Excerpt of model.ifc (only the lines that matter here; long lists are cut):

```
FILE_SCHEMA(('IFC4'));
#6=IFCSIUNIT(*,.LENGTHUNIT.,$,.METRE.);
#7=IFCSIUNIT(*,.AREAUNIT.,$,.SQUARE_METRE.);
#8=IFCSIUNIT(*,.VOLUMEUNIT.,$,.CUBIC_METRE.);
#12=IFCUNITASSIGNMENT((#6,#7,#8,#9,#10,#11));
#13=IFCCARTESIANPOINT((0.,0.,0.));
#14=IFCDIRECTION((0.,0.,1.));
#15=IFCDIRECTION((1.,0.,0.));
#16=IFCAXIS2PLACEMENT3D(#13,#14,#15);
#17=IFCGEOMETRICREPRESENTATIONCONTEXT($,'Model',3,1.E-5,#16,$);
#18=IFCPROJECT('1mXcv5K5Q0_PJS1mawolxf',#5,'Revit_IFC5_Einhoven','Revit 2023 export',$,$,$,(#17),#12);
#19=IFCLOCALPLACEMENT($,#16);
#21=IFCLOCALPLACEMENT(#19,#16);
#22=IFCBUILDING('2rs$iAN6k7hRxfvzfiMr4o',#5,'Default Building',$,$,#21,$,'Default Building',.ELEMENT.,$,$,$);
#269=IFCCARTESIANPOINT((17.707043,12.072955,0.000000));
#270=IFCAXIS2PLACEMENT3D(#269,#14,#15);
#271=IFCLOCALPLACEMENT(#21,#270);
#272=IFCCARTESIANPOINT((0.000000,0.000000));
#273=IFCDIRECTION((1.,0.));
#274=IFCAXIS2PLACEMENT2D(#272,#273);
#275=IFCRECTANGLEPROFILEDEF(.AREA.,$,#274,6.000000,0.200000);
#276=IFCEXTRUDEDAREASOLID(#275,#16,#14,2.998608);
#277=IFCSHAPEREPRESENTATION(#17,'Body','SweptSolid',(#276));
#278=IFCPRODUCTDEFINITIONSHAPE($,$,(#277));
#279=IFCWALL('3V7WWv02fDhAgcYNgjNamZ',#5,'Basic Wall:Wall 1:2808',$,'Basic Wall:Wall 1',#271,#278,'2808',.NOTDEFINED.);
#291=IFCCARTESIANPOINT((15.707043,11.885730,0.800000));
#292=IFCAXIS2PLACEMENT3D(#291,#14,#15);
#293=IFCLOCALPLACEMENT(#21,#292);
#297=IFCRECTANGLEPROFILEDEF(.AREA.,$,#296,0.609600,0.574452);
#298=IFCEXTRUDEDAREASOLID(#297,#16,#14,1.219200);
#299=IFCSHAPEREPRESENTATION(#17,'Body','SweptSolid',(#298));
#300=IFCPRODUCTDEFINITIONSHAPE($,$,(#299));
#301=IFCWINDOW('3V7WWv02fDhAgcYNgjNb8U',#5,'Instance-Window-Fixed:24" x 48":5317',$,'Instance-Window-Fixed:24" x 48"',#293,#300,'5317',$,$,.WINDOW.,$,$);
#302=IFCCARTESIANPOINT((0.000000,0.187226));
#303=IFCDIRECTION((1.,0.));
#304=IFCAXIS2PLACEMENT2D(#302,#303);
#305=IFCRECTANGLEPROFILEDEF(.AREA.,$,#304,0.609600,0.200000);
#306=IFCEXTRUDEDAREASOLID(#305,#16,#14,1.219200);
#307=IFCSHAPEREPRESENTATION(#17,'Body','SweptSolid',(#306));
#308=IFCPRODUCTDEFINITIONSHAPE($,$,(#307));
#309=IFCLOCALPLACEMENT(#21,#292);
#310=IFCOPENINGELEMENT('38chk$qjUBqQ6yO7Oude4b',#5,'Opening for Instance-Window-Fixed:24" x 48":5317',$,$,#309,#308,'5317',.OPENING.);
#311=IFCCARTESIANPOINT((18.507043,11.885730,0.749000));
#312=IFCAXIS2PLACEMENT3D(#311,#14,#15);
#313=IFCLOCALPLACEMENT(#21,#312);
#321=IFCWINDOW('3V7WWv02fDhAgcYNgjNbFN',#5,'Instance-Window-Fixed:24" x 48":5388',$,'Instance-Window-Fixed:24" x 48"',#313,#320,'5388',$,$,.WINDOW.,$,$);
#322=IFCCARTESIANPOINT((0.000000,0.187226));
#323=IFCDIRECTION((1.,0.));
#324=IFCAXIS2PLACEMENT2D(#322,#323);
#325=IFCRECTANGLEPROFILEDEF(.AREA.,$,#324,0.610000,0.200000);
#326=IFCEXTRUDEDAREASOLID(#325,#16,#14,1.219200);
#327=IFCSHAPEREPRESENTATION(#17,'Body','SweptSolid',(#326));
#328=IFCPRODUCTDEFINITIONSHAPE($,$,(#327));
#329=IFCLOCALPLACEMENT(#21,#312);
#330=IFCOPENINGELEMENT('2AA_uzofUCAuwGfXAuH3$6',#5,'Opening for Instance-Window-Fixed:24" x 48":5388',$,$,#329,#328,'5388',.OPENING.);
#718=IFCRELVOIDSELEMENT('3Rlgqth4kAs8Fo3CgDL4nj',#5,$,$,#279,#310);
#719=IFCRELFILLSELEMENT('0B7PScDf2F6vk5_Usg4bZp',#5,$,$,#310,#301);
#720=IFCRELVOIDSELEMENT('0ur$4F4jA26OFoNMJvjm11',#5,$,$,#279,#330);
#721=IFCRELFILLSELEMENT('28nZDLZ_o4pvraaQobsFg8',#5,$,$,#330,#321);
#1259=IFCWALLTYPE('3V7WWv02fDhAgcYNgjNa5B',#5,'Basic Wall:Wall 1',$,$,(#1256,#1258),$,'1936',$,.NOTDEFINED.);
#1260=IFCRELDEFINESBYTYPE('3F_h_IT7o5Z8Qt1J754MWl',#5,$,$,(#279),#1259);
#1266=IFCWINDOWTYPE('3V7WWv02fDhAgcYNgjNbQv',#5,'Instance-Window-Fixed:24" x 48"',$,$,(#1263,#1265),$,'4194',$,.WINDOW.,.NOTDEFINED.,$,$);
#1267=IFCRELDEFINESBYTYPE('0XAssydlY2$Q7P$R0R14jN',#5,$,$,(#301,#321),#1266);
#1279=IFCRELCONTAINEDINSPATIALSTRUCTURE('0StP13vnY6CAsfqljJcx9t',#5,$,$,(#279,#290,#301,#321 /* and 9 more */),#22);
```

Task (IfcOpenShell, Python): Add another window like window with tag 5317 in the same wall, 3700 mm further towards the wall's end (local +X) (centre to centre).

```python
import ifcopenshell
import ifcopenshell.api.feature
import ifcopenshell.api.geometry
import ifcopenshell.api.root
import ifcopenshell.geom
import ifcopenshell.util.element
import ifcopenshell.util.placement
import ifcopenshell.util.shape

model = ifcopenshell.open("model.ifc")
settings = ifcopenshell.geom.settings()


def volume(element):
    """Net volume in cubic metres, openings subtracted."""
    shape = ifcopenshell.geom.create_shape(settings, element)
    return ifcopenshell.util.shape.get_volume(shape.geometry)


def reuse_history(source, copy):
    """copy_class also copies each property set's owner history, people and application; keep the originals."""
    for rel in copy.IsDefinedBy:
        if rel.is_a("IfcRelDefinesByProperties") and (history := rel.RelatingPropertyDefinition.OwnerHistory):
            rel.RelatingPropertyDefinition.OwnerHistory = source.OwnerHistory
            ifcopenshell.util.element.remove_deep2(model, history)


window = model.by_guid("3V7WWv02fDhAgcYNgjNb8U")
opening = window.FillsVoids[0].RelatingOpeningElement
wall = opening.VoidsElements[0].RelatingBuildingElement
before = volume(wall)
shift = ifcopenshell.util.placement.get_local_placement(wall.ObjectPlacement)[:3, 0] * 3.7

# copy_class copies the void relationship, type, container and properties, but no geometry.
new_opening = ifcopenshell.api.root.copy_class(model, product=opening)
new_opening.Representation = ifcopenshell.util.element.copy_deep(
    model, opening.Representation, exclude=["IfcGeometricRepresentationContext", "IfcRepresentationMap"]
)
new_opening.Name = 'Opening for Instance-Window-Fixed:24" x 48"'
new_opening.Tag = None
new_window = ifcopenshell.api.root.copy_class(model, product=window)
new_window.Representation = ifcopenshell.util.element.copy_deep(
    model, window.Representation, exclude=["IfcGeometricRepresentationContext", "IfcRepresentationMap"]
)
new_window.Name = 'Instance-Window-Fixed:24" x 48"'
new_window.Tag = None
reuse_history(window, new_window)
ifcopenshell.api.feature.add_filling(model, opening=new_opening, element=new_window)

for old, new in ((opening, new_opening), (window, new_window)):
    matrix = ifcopenshell.util.placement.get_local_placement(old.ObjectPlacement)
    matrix[:3, 3] += shift
    ifcopenshell.api.geometry.edit_object_placement(model, product=new, matrix=matrix, is_si=False)

after = volume(wall)

print(f"wall volume {before:.3f} -> {after:.3f} m3")

model.write("model_v2.ifc")
```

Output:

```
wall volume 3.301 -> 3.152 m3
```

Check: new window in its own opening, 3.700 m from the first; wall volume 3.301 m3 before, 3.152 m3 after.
